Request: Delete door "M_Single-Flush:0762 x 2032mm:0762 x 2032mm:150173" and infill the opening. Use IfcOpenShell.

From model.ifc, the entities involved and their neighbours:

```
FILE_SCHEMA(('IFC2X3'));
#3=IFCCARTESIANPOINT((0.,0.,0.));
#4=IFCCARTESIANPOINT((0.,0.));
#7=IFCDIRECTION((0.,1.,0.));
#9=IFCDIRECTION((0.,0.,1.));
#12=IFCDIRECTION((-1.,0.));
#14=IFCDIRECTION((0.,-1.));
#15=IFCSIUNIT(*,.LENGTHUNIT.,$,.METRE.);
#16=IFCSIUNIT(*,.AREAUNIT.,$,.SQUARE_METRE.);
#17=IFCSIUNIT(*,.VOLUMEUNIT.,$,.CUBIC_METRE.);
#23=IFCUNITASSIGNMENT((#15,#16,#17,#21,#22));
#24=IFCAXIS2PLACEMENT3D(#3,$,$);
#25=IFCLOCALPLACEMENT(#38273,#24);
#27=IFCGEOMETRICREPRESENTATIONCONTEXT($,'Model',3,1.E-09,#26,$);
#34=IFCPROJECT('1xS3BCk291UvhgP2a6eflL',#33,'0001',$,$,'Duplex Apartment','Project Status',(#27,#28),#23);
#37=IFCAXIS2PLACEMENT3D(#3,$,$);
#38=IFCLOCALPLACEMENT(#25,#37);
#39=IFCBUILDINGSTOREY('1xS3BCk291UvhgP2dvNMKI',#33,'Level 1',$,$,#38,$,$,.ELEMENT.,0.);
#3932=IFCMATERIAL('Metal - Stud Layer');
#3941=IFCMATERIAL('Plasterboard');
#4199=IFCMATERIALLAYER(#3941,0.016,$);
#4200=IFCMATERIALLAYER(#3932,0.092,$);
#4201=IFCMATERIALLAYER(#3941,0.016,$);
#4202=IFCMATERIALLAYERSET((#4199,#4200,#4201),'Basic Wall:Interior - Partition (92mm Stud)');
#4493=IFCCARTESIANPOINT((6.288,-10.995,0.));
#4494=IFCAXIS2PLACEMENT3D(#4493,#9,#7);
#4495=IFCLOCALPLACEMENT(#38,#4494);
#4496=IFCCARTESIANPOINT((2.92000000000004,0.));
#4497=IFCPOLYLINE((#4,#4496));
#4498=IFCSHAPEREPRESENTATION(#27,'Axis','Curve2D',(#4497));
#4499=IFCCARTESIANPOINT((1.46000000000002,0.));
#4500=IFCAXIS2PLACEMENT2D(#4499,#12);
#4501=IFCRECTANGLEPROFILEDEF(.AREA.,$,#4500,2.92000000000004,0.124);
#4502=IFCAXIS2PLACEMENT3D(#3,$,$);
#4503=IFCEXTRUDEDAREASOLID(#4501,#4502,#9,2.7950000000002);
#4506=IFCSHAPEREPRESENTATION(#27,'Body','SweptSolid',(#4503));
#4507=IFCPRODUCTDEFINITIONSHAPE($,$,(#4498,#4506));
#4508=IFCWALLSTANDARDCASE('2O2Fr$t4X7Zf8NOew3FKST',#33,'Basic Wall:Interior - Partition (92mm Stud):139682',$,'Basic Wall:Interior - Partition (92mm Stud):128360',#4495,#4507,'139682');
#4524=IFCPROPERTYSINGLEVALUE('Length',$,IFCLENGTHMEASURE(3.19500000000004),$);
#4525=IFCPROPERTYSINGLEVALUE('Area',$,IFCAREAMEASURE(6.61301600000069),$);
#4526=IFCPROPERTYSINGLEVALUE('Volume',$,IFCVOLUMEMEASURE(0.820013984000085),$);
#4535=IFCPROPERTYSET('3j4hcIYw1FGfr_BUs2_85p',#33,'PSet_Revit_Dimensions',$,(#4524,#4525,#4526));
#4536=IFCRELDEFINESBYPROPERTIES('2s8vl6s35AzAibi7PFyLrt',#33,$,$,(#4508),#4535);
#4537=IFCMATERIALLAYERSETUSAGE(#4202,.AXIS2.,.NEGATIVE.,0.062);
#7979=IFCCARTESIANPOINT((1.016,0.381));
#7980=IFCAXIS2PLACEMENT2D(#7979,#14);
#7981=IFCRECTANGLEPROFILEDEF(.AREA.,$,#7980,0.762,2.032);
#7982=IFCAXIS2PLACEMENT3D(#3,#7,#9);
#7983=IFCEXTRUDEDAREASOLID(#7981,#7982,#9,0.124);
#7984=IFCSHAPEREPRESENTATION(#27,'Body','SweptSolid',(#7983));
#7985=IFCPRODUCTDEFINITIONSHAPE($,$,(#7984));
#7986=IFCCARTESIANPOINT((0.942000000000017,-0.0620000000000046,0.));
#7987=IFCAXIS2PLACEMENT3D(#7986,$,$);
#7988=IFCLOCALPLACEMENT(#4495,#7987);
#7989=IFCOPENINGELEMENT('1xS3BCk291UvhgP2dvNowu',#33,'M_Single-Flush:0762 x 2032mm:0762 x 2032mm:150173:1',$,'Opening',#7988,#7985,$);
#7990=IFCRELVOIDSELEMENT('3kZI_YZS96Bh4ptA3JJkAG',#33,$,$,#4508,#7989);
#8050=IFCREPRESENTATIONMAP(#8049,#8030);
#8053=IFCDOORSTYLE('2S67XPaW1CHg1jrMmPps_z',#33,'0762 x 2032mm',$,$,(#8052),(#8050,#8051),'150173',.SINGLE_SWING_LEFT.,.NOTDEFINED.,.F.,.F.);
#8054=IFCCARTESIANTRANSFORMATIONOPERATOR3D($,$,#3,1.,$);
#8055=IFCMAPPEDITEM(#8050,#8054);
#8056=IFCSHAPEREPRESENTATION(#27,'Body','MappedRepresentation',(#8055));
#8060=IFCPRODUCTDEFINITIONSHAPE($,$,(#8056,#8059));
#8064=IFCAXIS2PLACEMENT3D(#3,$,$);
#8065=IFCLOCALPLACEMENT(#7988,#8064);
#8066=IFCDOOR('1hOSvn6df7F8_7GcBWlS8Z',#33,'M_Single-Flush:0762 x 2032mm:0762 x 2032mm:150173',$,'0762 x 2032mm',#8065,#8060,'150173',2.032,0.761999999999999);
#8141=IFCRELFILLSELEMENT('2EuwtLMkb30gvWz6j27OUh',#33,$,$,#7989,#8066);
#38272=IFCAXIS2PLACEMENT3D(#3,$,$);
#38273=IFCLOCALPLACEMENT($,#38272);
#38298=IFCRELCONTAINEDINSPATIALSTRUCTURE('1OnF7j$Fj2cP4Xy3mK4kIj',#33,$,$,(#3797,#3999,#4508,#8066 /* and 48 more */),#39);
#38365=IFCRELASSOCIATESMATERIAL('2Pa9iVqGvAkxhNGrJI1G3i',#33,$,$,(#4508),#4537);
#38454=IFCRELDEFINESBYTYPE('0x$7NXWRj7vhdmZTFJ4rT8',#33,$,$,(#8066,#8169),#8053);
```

```python
import ifcopenshell
import ifcopenshell.api.feature
import ifcopenshell.api.pset
import ifcopenshell.api.root
import ifcopenshell.geom
import ifcopenshell.util.element
import ifcopenshell.util.shape
import ifcopenshell.util.unit

model = ifcopenshell.open("model.ifc")
area_scale = ifcopenshell.util.unit.calculate_unit_scale(model, "AREAUNIT")
volume_scale = ifcopenshell.util.unit.calculate_unit_scale(model, "VOLUMEUNIT")
settings = ifcopenshell.geom.settings()


def volume(element):
    """Net volume in cubic metres, openings subtracted."""
    shape = ifcopenshell.geom.create_shape(settings, element)
    return ifcopenshell.util.shape.get_volume(shape.geometry)


door = model.by_guid("1hOSvn6df7F8_7GcBWlS8Z")
opening = door.FillsVoids[0].RelatingOpeningElement
wall = opening.VoidsElements[0].RelatingBuildingElement
before = volume(wall)

ifcopenshell.api.root.remove_product(model, product=door)
ifcopenshell.api.feature.remove_feature(model, feature=opening)

after = volume(wall)
thickness = 0.124  # wall thickness in metres

# Update the wall's stored quantities.
pset = model.by_id(ifcopenshell.util.element.get_pset(wall, "PSet_Revit_Dimensions", should_inherit=False)["id"])
ifcopenshell.api.pset.edit_pset(model, pset=pset, properties={
    "Area": model.create_entity("IfcAreaMeasure", after / thickness / area_scale),
    "Volume": model.create_entity("IfcVolumeMeasure", after / volume_scale),
})

print(f"wall volume {before:.3f} -> {after:.3f} m3")

model.write("model-out.ifc")
```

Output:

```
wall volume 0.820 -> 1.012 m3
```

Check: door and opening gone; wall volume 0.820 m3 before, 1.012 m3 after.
